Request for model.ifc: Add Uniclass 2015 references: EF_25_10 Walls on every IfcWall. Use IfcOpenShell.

First a look at what the model holds.

```python
import ifcopenshell

model = ifcopenshell.open("model.ifc")
print(model.schema)
print("classifications:", [c.Name for c in model.by_type("IfcClassification")])
for ifc_class in ("IfcDoor", "IfcRoof", "IfcStair", "IfcWall", "IfcWindow"):
    print(ifc_class, len(model.by_type(ifc_class)))
```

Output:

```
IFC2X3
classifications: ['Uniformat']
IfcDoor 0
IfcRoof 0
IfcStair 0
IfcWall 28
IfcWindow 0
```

```python
import ifcopenshell
import ifcopenshell.api.classification

model = ifcopenshell.open("model.ifc")

# IFC2X3 requires Source and Edition and has no link from the project to the system.
system = model.create_entity("IfcClassification", Source="NBS", Edition="2015", Name="Uniclass 2015")

codes = {
    "IfcWall": ("EF_25_10", "Walls"),
}
for ifc_class, (code, name) in codes.items():
    products = model.by_type(ifc_class)
    ifcopenshell.api.classification.add_reference(
        model, products=products, classification=system, identification=code, name=name
    )
    print(code, len(products))

model.write("model_v2.ifc")
```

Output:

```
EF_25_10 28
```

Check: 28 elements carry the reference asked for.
